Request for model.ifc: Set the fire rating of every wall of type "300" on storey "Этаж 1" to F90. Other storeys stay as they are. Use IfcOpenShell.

First a look at what the model holds.

```python
import ifcopenshell
import ifcopenshell.util.element

model = ifcopenshell.open("model.ifc")
print(model.schema)
storey = next(s for s in model.by_type("IfcBuildingStorey") if s.Name == "Этаж 1")
walls = [e for e in ifcopenshell.util.element.get_decomposition(storey) if e.is_a("IfcWall")]
seen = {}
for e in walls:
    element_type = ifcopenshell.util.element.get_type(e)
    key = (element_type.Name if element_type != e and element_type else None, ifcopenshell.util.element.get_pset(e, "Pset_WallCommon", "FireRating"))
    seen[key] = seen.get(key, 0) + 1
for (name, value), count in sorted(seen.items(), key=str):
    print(count, "x", name, "|", value)
```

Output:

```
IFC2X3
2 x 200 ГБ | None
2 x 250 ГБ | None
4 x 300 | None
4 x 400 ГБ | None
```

```python
import ifcopenshell
import ifcopenshell.api.pset
import ifcopenshell.util.element

model = ifcopenshell.open("model.ifc")

storey = next(s for s in model.by_type("IfcBuildingStorey") if s.Name == "Этаж 1")
walls = [e for e in ifcopenshell.util.element.get_decomposition(storey) if e.is_a("IfcWall")]

count = 0
for e in walls:
    element_type = ifcopenshell.util.element.get_type(e)
    if element_type in (None, e) or element_type.Name != "300":
        continue
    # add_pset returns the element's existing set when there is one.
    pset = ifcopenshell.api.pset.add_pset(model, product=e, name="Pset_WallCommon")
    ifcopenshell.api.pset.edit_pset(model, pset=pset, properties={"FireRating": "F90"})
    count += 1

print(count, "walls updated")

model.write("model_v2.ifc")
```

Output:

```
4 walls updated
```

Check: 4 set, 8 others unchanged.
